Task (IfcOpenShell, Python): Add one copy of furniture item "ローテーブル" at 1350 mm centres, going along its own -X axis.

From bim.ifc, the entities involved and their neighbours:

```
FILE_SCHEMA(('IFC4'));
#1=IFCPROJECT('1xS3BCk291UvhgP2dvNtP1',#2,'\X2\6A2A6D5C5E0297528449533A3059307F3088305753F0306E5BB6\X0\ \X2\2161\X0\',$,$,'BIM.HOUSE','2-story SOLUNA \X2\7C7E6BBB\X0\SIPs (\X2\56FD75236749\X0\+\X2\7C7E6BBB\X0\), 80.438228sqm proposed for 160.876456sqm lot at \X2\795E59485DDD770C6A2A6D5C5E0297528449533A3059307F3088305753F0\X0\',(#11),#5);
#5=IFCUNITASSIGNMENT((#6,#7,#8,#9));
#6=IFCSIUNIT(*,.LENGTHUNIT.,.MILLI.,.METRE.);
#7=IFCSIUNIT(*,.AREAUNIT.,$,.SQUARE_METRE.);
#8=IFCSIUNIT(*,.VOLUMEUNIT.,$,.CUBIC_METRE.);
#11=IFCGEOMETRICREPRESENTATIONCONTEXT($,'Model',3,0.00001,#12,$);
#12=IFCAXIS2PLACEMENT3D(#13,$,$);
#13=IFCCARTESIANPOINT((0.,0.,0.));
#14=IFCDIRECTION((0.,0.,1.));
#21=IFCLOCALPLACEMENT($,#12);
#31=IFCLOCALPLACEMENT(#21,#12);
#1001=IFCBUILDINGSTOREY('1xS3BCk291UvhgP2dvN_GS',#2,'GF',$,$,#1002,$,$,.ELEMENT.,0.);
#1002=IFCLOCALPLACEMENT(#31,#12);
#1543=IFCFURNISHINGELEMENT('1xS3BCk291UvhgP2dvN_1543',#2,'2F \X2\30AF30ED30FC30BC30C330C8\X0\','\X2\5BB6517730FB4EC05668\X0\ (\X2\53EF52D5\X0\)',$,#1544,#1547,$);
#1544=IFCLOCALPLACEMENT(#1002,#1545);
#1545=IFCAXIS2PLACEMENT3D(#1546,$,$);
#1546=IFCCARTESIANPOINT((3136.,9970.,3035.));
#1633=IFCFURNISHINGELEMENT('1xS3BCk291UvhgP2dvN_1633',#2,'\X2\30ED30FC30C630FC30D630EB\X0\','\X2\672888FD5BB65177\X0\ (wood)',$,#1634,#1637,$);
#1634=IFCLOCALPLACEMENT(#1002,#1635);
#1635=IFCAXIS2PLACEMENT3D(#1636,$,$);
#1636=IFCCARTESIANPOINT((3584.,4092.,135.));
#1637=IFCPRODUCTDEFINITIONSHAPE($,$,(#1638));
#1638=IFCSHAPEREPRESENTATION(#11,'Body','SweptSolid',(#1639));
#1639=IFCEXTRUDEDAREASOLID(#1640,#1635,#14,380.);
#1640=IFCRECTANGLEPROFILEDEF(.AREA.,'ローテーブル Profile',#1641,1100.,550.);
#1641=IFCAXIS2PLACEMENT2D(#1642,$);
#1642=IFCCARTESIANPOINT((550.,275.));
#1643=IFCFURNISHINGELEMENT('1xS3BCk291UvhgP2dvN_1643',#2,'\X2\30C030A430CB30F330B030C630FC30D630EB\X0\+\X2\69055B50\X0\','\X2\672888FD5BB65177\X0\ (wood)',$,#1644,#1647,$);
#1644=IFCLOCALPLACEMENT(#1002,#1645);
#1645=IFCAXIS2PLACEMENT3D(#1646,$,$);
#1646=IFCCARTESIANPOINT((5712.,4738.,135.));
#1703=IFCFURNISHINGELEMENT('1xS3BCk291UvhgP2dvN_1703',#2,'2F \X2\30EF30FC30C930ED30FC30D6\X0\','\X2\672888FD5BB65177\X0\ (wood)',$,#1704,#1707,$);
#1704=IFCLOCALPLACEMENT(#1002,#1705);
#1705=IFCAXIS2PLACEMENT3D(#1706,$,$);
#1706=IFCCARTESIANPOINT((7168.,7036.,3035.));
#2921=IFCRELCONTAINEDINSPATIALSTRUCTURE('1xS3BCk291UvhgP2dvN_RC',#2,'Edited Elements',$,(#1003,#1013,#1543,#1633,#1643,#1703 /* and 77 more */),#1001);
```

```python
import ifcopenshell
import ifcopenshell.api.geometry
import ifcopenshell.api.root
import ifcopenshell.util.element
import ifcopenshell.util.placement
import ifcopenshell.util.unit

model = ifcopenshell.open("bim.ifc")
unit_scale = ifcopenshell.util.unit.calculate_unit_scale(model)


def reuse_history(source, copy):
    """copy_class also copies each property set's owner history, people and application; keep the originals."""
    for rel in copy.IsDefinedBy:
        if rel.is_a("IfcRelDefinesByProperties") and (history := rel.RelatingPropertyDefinition.OwnerHistory):
            rel.RelatingPropertyDefinition.OwnerHistory = source.OwnerHistory
            ifcopenshell.util.element.remove_deep2(model, history)


source = model.by_guid("1xS3BCk291UvhgP2dvN_1633")
base = ifcopenshell.util.placement.get_local_placement(source.ObjectPlacement)
step = -base[:3, 0] * 1.35 / unit_scale

for i in range(1, 2):
    copy = ifcopenshell.api.root.copy_class(model, product=source)
    copy.Representation = ifcopenshell.util.element.copy_deep(
        model, source.Representation, exclude=["IfcGeometricRepresentationContext", "IfcRepresentationMap"]
    )
    reuse_history(source, copy)
    matrix = base.copy()
    matrix[:3, 3] += i * step
    print("added at", matrix[:3, 3].round(3) + 0.0)
    ifcopenshell.api.geometry.edit_object_placement(model, product=copy, matrix=matrix, is_si=False)

model.write("bim_updated.ifc")
```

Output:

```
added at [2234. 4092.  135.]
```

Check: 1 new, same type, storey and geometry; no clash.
